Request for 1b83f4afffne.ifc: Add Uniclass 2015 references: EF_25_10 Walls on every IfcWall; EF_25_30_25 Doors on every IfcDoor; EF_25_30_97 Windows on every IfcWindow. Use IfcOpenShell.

First a look at what the model holds.

```python
import ifcopenshell

model = ifcopenshell.open("1b83f4afffne.ifc")
print(model.schema)
print("classifications:", [c.Name for c in model.by_type("IfcClassification")])
for ifc_class in ("IfcDoor", "IfcRoof", "IfcStair", "IfcWall", "IfcWindow"):
    print(ifc_class, len(model.by_type(ifc_class)))
```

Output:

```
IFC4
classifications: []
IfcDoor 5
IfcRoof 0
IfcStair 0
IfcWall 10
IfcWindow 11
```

```python
import ifcopenshell
import ifcopenshell.api.classification

model = ifcopenshell.open("1b83f4afffne.ifc")

system = ifcopenshell.api.classification.add_classification(model, classification="Uniclass 2015")

codes = {
    "IfcWall": ("EF_25_10", "Walls"),
    "IfcDoor": ("EF_25_30_25", "Doors"),
    "IfcWindow": ("EF_25_30_97", "Windows"),
}
for ifc_class, (code, name) in codes.items():
    products = model.by_type(ifc_class)
    ifcopenshell.api.classification.add_reference(
        model, products=products, classification=system, identification=code, name=name
    )
    print(code, len(products))

model.write("1b83f4afffne_updated.ifc")
```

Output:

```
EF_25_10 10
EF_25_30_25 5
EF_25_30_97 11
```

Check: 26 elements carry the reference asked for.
